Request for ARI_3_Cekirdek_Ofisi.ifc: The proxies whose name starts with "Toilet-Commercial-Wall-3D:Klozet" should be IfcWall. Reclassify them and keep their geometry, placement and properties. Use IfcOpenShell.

First a look at what the model holds.

```python
import re

import ifcopenshell

model = ifcopenshell.open("ARI_3_Cekirdek_Ofisi.ifc")
print(model.schema)
seen = {}
for e in model.by_type("IfcBuildingElementProxy"):
    name = re.sub(r":\d+(:\d+)?$", "", e.Name or "")  # drop the element id that some exporters append
    seen[name] = seen.get(name, 0) + 1
for name, count in sorted(seen.items()):
    print(count, "x", name)
```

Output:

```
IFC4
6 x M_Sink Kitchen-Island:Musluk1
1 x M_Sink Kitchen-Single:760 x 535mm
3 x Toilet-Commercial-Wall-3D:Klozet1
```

```python
import ifcopenshell
import ifcopenshell.api.root

model = ifcopenshell.open("ARI_3_Cekirdek_Ofisi.ifc")

proxies = [e.id() for e in model.by_type("IfcBuildingElementProxy") if (e.Name or "").startswith("Toilet-Commercial-Wall-3D:Klozet")]
for step_id in proxies:
    proxy = model.by_id(step_id)
    ifcopenshell.api.root.reassign_class(model, product=proxy, ifc_class="IfcWall")

print(sum(model.by_id(i).is_a("IfcWall") for i in proxies), "reclassified")

model.write("ARI_3_Cekirdek_Ofisi_updated.ifc")
```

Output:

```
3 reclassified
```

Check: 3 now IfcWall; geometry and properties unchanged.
